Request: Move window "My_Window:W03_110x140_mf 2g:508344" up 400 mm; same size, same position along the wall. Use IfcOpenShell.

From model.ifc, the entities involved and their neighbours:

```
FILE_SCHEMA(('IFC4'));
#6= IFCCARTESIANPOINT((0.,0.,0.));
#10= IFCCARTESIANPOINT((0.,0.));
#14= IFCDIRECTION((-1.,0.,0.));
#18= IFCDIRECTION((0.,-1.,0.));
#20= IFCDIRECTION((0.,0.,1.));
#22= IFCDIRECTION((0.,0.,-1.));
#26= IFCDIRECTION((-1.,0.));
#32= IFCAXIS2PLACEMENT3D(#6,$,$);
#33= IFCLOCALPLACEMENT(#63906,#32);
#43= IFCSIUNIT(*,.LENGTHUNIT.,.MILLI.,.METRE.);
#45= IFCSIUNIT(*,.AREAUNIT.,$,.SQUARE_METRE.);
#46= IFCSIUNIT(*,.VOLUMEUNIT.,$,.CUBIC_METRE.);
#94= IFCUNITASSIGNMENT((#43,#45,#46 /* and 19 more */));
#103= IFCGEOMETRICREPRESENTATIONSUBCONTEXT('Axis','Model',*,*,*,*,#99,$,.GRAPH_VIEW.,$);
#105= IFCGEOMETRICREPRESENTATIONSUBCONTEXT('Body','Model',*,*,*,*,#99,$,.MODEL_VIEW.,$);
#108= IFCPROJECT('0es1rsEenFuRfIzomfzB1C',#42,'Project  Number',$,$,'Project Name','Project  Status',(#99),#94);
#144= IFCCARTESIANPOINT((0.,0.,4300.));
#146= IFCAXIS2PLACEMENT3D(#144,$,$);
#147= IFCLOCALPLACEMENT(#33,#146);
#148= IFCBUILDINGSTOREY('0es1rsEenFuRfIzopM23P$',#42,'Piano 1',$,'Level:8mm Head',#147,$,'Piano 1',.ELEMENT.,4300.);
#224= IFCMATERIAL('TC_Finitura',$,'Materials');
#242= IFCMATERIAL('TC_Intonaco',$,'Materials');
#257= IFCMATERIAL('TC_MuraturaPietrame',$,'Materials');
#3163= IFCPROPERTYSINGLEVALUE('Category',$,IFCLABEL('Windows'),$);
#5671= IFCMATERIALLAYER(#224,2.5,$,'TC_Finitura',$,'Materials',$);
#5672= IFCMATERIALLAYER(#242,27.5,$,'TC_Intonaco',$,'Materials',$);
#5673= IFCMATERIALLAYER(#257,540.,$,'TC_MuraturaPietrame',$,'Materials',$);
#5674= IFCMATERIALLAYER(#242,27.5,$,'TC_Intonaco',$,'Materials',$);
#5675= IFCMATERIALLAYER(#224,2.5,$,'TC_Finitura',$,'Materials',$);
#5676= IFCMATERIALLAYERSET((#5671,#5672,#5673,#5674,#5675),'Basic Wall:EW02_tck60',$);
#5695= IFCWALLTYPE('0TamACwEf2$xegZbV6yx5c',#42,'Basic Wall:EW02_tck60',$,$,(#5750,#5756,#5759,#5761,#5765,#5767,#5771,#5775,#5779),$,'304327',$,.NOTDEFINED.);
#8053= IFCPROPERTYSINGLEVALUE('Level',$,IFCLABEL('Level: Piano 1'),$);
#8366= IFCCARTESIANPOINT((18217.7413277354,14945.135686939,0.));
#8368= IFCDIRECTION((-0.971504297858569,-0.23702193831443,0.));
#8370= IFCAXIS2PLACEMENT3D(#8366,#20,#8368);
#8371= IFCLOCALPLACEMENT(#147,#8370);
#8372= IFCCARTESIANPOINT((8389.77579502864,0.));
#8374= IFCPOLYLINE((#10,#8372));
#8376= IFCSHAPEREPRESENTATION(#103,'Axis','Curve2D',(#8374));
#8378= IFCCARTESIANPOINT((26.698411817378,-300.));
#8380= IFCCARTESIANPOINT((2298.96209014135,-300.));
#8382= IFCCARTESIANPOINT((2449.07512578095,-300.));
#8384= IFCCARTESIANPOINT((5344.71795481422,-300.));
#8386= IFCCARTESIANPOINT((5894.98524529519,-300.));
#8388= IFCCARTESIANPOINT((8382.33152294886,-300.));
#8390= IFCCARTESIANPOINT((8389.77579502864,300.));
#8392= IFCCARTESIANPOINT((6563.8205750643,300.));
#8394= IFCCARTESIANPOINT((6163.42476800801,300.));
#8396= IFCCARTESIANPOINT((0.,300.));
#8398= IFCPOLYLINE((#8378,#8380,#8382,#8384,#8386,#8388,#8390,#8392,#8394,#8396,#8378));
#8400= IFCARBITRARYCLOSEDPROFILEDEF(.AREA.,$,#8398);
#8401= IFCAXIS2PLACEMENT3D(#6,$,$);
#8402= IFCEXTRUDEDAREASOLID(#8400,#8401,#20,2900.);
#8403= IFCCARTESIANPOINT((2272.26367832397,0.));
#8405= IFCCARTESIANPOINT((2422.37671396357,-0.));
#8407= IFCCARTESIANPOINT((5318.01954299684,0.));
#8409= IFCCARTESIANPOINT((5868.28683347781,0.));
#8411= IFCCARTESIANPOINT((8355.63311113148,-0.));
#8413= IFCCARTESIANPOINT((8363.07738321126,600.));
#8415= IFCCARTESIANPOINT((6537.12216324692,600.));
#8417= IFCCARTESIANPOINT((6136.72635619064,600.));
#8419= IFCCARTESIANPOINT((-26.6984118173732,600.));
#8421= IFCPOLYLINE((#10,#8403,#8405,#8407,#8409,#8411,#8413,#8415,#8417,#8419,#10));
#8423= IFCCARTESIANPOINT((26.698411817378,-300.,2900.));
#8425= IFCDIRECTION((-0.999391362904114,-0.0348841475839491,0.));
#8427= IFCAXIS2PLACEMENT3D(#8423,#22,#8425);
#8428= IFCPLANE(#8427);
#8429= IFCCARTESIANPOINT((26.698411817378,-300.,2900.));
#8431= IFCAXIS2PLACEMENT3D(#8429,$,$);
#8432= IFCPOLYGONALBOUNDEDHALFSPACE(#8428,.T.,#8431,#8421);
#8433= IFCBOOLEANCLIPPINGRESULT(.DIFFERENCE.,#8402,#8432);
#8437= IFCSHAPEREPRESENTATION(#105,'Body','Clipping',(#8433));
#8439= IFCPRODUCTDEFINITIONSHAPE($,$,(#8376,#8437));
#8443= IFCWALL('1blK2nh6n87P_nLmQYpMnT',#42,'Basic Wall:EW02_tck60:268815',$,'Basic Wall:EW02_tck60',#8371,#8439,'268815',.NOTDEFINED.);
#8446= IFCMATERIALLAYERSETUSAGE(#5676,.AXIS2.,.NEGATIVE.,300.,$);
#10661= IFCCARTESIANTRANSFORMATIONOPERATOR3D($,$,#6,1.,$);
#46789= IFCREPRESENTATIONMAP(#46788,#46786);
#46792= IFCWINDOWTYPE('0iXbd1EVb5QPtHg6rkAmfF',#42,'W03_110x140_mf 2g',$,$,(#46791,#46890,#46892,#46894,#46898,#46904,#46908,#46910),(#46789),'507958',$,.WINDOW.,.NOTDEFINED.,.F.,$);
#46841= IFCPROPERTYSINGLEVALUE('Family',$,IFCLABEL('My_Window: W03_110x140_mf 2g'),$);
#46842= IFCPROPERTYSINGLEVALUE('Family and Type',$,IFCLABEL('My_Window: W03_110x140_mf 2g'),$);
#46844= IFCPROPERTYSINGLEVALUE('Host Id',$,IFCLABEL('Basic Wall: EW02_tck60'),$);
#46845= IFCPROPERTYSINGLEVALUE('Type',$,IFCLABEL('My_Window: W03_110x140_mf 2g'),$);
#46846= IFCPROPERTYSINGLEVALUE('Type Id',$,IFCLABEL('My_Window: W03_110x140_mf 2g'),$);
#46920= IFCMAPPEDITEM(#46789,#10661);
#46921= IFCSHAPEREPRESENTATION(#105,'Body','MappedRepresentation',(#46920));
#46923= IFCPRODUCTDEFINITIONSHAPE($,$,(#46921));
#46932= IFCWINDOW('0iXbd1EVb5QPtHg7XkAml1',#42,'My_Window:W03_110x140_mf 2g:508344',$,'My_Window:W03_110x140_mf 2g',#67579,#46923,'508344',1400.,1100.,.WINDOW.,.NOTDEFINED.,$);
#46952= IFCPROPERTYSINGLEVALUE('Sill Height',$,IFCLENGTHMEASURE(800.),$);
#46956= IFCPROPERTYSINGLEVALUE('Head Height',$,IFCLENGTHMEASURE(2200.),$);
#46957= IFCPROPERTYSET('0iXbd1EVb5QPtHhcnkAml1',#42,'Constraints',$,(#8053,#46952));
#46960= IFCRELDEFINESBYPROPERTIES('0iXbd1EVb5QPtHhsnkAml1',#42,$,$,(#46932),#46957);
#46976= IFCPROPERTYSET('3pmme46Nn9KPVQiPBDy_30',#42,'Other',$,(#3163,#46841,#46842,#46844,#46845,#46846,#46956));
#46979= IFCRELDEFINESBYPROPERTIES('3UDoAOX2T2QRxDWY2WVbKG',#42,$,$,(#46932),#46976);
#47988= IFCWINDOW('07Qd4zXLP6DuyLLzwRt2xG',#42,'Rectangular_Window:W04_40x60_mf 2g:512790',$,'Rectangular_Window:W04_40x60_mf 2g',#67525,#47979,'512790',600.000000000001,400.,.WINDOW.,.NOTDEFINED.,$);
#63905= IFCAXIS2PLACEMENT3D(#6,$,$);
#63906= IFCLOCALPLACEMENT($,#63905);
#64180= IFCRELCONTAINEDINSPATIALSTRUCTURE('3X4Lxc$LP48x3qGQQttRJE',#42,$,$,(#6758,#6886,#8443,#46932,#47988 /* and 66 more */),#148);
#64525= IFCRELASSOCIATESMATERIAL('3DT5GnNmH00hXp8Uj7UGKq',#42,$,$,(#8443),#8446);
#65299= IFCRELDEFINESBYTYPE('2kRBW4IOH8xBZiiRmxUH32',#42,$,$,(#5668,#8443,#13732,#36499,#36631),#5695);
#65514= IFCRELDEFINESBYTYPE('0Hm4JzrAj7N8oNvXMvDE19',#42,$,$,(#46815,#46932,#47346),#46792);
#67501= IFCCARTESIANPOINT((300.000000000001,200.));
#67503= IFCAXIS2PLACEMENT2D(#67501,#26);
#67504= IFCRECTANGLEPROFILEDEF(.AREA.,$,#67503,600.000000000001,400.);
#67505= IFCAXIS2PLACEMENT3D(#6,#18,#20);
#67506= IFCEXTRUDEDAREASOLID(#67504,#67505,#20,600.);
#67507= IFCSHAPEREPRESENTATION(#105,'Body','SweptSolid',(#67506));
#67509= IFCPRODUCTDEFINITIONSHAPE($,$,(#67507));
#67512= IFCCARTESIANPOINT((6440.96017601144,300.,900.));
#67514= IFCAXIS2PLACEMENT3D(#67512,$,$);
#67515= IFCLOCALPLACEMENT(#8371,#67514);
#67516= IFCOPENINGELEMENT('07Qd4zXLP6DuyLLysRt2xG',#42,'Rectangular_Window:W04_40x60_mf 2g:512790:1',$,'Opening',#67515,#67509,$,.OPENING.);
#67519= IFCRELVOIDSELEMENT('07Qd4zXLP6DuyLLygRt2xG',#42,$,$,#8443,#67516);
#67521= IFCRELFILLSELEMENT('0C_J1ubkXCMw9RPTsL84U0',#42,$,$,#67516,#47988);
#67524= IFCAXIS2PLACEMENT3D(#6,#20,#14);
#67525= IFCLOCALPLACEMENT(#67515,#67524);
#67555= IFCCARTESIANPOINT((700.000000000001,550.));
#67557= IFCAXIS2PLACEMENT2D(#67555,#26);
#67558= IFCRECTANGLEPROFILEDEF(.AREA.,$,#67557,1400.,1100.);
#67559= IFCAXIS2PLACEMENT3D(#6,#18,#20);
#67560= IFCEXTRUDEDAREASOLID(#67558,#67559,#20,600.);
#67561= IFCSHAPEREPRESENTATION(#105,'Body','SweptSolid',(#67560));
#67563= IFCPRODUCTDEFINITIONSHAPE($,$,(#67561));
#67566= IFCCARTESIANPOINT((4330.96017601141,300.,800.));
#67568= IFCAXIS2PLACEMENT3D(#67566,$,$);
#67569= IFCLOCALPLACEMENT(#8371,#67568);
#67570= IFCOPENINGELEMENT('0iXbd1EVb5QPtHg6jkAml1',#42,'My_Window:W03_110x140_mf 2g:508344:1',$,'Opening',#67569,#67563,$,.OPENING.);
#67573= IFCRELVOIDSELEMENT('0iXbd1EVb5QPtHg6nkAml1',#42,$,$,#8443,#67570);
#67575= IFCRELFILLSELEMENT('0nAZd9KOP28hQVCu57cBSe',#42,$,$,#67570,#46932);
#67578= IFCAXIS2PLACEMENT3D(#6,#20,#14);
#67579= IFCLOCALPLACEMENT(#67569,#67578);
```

```python
import numpy as np
import ifcopenshell
import ifcopenshell.api.geometry
import ifcopenshell.api.pset
import ifcopenshell.util.element
import ifcopenshell.util.placement
import ifcopenshell.util.unit

model = ifcopenshell.open("model.ifc")
unit_scale = ifcopenshell.util.unit.calculate_unit_scale(model)

window = model.by_id(46932)
opening = window.FillsVoids[0].RelatingOpeningElement
dz = 400.0

shift = np.array([0.0, 0.0, dz])
# The window is placed relative to its opening, so it follows when the opening moves.
matrix = ifcopenshell.util.placement.get_local_placement(opening.ObjectPlacement)
matrix[:3, 3] += shift
ifcopenshell.api.geometry.edit_object_placement(
    model, product=opening, matrix=matrix, is_si=False, should_transform_children=True
)

# Keep the stored heights in step.
pset = model.by_id(ifcopenshell.util.element.get_pset(window, "Constraints", should_inherit=False)["id"])
ifcopenshell.api.pset.edit_pset(model, pset=pset, properties={
    "Sill Height": model.create_entity("IfcLengthMeasure", ifcopenshell.util.element.get_pset(window, "Constraints", "Sill Height") + dz),
})
pset = model.by_id(ifcopenshell.util.element.get_pset(window, "Other", should_inherit=False)["id"])
ifcopenshell.api.pset.edit_pset(model, pset=pset, properties={
    "Head Height": model.create_entity("IfcLengthMeasure", ifcopenshell.util.element.get_pset(window, "Other", "Head Height") + dz),
})

print(f"moved by {dz * unit_scale:+.3f} m")

model.write("model_rev.ifc")
```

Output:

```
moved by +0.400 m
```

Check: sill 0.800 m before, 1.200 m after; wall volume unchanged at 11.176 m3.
